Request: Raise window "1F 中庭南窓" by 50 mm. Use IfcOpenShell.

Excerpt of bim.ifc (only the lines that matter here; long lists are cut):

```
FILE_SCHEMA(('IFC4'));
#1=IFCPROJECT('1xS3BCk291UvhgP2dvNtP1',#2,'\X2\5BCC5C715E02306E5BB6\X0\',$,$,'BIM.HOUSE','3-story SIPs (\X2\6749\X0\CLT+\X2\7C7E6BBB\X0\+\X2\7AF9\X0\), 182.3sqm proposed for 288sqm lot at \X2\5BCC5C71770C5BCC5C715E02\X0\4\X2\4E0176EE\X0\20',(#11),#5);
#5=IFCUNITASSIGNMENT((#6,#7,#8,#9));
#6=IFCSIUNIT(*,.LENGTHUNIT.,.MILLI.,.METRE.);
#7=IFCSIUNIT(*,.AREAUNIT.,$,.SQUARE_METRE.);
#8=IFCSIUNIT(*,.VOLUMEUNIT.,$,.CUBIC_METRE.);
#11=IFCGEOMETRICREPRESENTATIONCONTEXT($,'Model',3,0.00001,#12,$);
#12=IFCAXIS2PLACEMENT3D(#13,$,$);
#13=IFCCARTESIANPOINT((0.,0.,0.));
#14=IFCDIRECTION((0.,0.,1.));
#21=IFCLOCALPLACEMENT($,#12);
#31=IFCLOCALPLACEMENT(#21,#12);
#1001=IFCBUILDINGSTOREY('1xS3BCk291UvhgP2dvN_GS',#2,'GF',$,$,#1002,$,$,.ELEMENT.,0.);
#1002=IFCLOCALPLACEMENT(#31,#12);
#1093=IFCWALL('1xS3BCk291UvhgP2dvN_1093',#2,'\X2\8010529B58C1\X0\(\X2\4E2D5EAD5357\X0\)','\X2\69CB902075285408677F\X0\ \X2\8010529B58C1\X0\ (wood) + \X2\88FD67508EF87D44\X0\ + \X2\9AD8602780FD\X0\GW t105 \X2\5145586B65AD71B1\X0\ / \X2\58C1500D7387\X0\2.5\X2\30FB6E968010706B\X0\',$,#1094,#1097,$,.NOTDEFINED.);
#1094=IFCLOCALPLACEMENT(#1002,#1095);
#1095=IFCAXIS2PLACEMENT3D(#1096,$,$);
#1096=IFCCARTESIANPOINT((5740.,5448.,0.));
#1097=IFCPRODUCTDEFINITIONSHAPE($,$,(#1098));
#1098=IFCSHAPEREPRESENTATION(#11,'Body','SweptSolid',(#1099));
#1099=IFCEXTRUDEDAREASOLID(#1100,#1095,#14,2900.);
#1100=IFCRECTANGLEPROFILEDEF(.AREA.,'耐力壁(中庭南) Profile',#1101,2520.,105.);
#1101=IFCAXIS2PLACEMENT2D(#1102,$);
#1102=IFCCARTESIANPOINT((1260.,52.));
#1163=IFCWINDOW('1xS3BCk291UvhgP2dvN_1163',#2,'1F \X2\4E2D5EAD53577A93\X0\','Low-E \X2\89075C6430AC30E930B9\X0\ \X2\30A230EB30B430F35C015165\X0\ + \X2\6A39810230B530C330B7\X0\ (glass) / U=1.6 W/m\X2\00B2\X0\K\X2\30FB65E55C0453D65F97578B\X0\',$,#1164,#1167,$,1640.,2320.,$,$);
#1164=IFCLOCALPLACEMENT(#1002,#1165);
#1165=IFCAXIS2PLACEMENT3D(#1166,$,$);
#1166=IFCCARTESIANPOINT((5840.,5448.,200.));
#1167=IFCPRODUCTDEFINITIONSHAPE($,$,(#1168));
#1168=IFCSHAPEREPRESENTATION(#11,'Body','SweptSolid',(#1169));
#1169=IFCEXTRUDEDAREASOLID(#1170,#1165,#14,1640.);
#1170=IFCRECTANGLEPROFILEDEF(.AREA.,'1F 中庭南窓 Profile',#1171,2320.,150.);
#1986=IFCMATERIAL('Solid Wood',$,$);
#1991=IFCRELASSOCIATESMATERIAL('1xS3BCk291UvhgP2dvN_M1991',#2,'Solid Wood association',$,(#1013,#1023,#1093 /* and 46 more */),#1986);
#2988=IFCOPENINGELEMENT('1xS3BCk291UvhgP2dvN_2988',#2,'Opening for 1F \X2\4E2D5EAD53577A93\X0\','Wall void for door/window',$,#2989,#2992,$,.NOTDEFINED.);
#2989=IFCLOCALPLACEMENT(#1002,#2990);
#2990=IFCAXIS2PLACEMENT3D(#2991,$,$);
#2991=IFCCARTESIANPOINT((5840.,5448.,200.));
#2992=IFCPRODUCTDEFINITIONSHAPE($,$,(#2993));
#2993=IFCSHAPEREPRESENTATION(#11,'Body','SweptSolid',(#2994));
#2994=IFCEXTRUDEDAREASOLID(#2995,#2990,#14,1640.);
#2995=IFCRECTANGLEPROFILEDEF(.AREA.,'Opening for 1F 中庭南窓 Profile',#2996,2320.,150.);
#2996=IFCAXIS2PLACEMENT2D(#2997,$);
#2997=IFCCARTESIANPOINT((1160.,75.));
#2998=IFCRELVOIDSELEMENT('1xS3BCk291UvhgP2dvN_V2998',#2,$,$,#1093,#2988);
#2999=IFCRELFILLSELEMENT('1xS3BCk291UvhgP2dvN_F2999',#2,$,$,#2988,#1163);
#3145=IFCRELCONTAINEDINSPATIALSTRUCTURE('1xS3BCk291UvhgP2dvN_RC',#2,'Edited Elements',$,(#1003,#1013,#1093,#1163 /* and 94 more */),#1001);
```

```python
import numpy as np
import ifcopenshell
import ifcopenshell.api.geometry
import ifcopenshell.util.placement
import ifcopenshell.util.unit

model = ifcopenshell.open("bim.ifc")
unit_scale = ifcopenshell.util.unit.calculate_unit_scale(model)

window = model.by_guid("1xS3BCk291UvhgP2dvN_1163")
opening = window.FillsVoids[0].RelatingOpeningElement
dz = 0.05 / unit_scale

shift = np.array([0.0, 0.0, dz])
# The window is not placed relative to its opening, so move both.
for product in (opening, window):
    matrix = ifcopenshell.util.placement.get_local_placement(product.ObjectPlacement)
    matrix[:3, 3] += shift
    ifcopenshell.api.geometry.edit_object_placement(model, product=product, matrix=matrix, is_si=False)

print(f"moved by {dz * unit_scale:+.3f} m")

model.write("bim-out.ifc")
```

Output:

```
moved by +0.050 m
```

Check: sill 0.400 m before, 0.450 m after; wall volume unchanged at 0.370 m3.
